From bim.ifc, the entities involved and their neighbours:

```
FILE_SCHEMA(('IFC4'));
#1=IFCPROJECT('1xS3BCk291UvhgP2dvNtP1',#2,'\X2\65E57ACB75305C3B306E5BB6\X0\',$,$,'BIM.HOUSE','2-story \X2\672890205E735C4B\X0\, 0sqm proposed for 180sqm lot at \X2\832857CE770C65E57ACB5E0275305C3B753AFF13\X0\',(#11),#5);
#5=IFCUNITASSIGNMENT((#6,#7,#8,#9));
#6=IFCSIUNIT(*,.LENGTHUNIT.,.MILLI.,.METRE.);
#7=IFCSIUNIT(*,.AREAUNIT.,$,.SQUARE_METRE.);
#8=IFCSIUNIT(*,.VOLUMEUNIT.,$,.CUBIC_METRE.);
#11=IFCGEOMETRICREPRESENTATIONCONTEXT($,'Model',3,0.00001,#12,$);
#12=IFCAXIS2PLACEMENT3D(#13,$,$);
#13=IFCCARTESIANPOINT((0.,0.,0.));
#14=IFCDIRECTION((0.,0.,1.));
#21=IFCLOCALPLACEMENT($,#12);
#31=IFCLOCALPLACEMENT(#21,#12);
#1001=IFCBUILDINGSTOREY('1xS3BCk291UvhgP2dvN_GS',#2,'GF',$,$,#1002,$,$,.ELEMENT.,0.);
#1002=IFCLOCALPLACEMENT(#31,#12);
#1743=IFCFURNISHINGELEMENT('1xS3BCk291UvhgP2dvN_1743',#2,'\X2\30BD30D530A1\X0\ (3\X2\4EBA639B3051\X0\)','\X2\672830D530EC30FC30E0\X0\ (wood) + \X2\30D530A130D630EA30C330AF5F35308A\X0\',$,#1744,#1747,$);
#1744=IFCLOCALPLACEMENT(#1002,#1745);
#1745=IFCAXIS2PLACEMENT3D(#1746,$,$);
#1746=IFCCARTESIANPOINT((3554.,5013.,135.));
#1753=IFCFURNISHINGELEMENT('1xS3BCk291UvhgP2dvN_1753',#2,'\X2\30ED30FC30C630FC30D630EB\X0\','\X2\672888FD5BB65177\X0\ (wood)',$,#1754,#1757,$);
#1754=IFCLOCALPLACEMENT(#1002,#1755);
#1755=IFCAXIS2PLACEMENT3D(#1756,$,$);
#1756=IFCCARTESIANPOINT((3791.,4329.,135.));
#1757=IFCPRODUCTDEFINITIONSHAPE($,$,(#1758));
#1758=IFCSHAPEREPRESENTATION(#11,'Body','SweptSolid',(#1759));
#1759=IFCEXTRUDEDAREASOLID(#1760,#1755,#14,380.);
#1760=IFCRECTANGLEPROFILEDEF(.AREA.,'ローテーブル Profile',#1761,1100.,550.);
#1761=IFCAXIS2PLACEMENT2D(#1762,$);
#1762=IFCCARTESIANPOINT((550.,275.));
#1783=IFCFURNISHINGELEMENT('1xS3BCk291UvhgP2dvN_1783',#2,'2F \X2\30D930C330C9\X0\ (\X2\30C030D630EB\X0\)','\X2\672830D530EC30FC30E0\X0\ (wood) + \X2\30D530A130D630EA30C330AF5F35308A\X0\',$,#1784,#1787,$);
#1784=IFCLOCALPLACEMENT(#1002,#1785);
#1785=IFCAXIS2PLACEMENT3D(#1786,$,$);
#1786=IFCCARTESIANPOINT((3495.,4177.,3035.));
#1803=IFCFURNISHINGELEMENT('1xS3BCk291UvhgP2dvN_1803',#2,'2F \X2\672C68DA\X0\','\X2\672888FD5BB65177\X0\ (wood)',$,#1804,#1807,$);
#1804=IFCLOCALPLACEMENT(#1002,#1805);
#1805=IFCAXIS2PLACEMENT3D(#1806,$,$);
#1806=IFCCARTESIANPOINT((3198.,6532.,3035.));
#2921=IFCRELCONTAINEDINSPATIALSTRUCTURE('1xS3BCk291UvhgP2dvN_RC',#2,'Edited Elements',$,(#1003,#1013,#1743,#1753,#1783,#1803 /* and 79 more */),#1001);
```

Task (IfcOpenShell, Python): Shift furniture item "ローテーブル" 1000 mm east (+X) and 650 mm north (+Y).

```python
import ifcopenshell
import ifcopenshell.api.geometry
import ifcopenshell.util.placement

model = ifcopenshell.open("bim.ifc")

item = model.by_guid("1xS3BCk291UvhgP2dvN_1753")
matrix = ifcopenshell.util.placement.get_local_placement(item.ObjectPlacement)
matrix[0, 3] += 1000.0
matrix[1, 3] += 650.0
ifcopenshell.api.geometry.edit_object_placement(model, product=item, matrix=matrix, is_si=False)

print(ifcopenshell.util.placement.get_local_placement(item.ObjectPlacement).round(3) + 0.0)

model.write("bim_edited.ifc")
```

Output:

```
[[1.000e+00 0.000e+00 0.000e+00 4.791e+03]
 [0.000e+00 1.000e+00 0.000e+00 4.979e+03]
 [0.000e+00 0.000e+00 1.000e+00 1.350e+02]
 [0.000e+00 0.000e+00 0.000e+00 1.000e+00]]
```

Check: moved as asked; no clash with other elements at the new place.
